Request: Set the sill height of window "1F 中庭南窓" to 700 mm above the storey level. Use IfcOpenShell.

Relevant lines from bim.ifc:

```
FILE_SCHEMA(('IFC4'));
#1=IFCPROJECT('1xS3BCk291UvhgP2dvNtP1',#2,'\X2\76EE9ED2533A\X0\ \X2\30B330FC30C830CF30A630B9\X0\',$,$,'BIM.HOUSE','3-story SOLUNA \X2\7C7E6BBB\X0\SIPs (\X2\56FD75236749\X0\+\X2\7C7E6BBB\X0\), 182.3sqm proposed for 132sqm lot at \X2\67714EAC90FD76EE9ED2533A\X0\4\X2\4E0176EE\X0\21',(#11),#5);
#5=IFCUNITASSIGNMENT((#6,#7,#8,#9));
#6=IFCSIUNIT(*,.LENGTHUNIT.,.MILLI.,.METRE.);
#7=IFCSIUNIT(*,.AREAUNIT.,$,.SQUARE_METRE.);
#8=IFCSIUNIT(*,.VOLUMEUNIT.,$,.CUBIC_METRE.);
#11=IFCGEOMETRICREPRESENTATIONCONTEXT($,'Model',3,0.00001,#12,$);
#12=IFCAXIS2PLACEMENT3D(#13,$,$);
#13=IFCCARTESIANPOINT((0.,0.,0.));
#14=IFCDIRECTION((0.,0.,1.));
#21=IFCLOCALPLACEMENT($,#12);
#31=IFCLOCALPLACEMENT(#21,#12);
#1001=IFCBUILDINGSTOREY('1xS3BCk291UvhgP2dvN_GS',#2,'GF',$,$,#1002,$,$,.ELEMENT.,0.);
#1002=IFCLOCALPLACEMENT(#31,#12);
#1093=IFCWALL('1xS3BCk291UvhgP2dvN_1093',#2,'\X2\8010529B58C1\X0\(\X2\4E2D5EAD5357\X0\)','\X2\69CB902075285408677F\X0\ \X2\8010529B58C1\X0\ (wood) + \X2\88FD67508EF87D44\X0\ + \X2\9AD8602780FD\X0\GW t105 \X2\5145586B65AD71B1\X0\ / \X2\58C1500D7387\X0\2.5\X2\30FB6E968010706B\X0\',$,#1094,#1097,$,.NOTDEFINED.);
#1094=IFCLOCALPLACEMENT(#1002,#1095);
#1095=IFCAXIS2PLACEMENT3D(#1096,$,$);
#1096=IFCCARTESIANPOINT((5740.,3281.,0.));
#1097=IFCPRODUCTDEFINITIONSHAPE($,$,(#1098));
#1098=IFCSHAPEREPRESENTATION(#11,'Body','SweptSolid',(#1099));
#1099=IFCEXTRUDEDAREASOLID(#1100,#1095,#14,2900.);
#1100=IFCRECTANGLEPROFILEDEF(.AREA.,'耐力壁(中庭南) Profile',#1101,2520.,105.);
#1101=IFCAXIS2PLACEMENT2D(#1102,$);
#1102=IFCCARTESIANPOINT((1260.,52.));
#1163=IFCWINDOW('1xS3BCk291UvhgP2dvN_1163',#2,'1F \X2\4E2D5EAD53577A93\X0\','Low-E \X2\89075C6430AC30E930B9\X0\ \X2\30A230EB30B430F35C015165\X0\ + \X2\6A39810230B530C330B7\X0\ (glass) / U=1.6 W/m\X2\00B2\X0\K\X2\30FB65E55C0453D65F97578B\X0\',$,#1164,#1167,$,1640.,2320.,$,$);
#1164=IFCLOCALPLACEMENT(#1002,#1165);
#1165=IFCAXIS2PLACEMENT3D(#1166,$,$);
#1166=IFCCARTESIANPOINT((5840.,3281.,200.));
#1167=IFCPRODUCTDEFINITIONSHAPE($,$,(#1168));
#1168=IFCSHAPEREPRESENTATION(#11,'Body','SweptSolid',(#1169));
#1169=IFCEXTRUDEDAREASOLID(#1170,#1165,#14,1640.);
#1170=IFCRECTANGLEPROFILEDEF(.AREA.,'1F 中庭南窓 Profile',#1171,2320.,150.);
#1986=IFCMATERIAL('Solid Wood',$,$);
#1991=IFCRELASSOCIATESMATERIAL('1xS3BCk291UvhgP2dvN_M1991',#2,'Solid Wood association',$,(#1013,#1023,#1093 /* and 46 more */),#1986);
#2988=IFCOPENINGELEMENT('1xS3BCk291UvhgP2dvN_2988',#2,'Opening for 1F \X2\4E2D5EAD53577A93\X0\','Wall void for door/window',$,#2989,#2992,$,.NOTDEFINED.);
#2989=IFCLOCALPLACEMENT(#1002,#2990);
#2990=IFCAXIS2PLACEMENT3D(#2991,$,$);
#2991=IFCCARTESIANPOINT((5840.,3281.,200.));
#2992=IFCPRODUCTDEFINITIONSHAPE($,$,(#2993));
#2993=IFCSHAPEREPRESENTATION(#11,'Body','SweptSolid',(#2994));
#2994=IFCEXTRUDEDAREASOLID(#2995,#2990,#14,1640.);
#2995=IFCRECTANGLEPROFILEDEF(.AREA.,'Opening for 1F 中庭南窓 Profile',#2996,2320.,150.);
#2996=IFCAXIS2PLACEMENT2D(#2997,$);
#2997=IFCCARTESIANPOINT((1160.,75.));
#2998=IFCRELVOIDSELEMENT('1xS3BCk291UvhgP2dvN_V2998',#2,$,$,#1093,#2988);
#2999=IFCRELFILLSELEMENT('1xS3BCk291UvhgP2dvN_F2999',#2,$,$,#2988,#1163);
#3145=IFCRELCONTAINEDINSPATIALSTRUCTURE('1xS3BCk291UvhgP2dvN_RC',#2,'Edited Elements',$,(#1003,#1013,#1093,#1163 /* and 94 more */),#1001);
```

```python
import numpy as np
import ifcopenshell
import ifcopenshell.api.geometry
import ifcopenshell.geom
import ifcopenshell.util.element
import ifcopenshell.util.placement
import ifcopenshell.util.shape
import ifcopenshell.util.unit

model = ifcopenshell.open("bim.ifc")
unit_scale = ifcopenshell.util.unit.calculate_unit_scale(model)

window = model.by_guid("1xS3BCk291UvhgP2dvN_1163")
opening = window.FillsVoids[0].RelatingOpeningElement
storey = ifcopenshell.util.element.get_container(window, ifc_class="IfcBuildingStorey")
level = ifcopenshell.util.placement.get_local_placement(storey.ObjectPlacement)[2, 3]

# The opening's origin need not be at the sill, so measure its lowest point.
shape = ifcopenshell.geom.create_shape(ifcopenshell.geom.settings(), opening)
bottom = ifcopenshell.util.shape.get_shape_bottom_elevation(shape, shape.geometry) / unit_scale
dz = level + 0.7 / unit_scale - bottom

shift = np.array([0.0, 0.0, dz])
# The window is not placed relative to its opening, so move both.
for product in (opening, window):
    matrix = ifcopenshell.util.placement.get_local_placement(product.ObjectPlacement)
    matrix[:3, 3] += shift
    ifcopenshell.api.geometry.edit_object_placement(model, product=product, matrix=matrix, is_si=False)

print(f"moved by {dz * unit_scale:+.3f} m")

model.write("bim_edited.ifc")
```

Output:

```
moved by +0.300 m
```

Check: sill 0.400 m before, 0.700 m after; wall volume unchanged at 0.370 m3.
